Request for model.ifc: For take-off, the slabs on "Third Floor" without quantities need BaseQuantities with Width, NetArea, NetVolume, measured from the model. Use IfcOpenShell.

First a look at what the model holds.

```python
import ifcopenshell
import ifcopenshell.util.element
import ifcopenshell.util.unit

model = ifcopenshell.open("model.ifc")
print(model.schema)
for unit_type in ("LENGTHUNIT", "AREAUNIT", "VOLUMEUNIT"):
    print(unit_type, ifcopenshell.util.unit.calculate_unit_scale(model, unit_type))
storey = next(s for s in model.by_type("IfcBuildingStorey") if s.Name == "Third Floor")
slabs = [e for e in ifcopenshell.util.element.get_decomposition(storey) if e.is_a("IfcSlab")]
for e in sorted(slabs, key=lambda e: e.id()):
    print(e.id(), e.is_a(), e.Name, list(ifcopenshell.util.element.get_psets(e, qtos_only=True)), sep=" | ")
```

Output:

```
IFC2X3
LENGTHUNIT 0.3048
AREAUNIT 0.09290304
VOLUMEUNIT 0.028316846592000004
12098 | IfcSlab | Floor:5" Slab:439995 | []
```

```python
import ifcopenshell
import ifcopenshell.api.pset
import ifcopenshell.geom
import ifcopenshell.util.element
import ifcopenshell.util.shape
import ifcopenshell.util.unit

model = ifcopenshell.open("model.ifc")
unit_scale = ifcopenshell.util.unit.calculate_unit_scale(model)
area_scale = ifcopenshell.util.unit.calculate_unit_scale(model, "AREAUNIT")
volume_scale = ifcopenshell.util.unit.calculate_unit_scale(model, "VOLUMEUNIT")
settings = ifcopenshell.geom.settings()

storey = next(s for s in model.by_type("IfcBuildingStorey") if s.Name == "Third Floor")
slabs = [e for e in ifcopenshell.util.element.get_decomposition(storey) if e.is_a("IfcSlab")]

for e in sorted(slabs, key=lambda e: e.id()):
    if ifcopenshell.util.element.get_psets(e, qtos_only=True, should_inherit=False):
        continue
    # Geometry comes back in metres, in the element's own axes.
    shape = ifcopenshell.geom.create_shape(settings, e)
    values = {
        "Width": ifcopenshell.util.shape.get_z(shape.geometry) / unit_scale,
        "NetArea": ifcopenshell.util.shape.get_footprint_area(shape.geometry) / area_scale,
        "NetVolume": ifcopenshell.util.shape.get_volume(shape.geometry) / volume_scale,
    }
    qto = ifcopenshell.api.pset.add_qto(model, product=e, name="BaseQuantities")
    ifcopenshell.api.pset.edit_qto(model, qto=qto, properties=values)
    print(e.id(), {k: round(v, 3) for k, v in values.items()})

model.write("model_edited.ifc")
```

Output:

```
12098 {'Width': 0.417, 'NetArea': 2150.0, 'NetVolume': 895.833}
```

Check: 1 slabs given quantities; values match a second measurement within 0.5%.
